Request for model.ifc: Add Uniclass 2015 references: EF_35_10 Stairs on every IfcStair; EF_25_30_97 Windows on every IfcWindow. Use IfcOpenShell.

First a look at what the model holds.

```python
import ifcopenshell

model = ifcopenshell.open("model.ifc")
print(model.schema)
print("classifications:", [c.Name for c in model.by_type("IfcClassification")])
for ifc_class in ("IfcDoor", "IfcRoof", "IfcStair", "IfcWall", "IfcWindow"):
    print(ifc_class, len(model.by_type(ifc_class)))
```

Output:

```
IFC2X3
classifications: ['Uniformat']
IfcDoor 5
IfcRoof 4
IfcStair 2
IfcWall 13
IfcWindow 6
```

```python
import ifcopenshell
import ifcopenshell.api.classification

model = ifcopenshell.open("model.ifc")

# IFC2X3 requires Source and Edition and has no link from the project to the system.
system = model.create_entity("IfcClassification", Source="NBS", Edition="2015", Name="Uniclass 2015")

codes = {
    "IfcStair": ("EF_35_10", "Stairs"),
    "IfcWindow": ("EF_25_30_97", "Windows"),
}
for ifc_class, (code, name) in codes.items():
    products = model.by_type(ifc_class)
    ifcopenshell.api.classification.add_reference(
        model, products=products, classification=system, identification=code, name=name
    )
    print(code, len(products))

model.write("model_rev.ifc")
```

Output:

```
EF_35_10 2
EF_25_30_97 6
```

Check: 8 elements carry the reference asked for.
